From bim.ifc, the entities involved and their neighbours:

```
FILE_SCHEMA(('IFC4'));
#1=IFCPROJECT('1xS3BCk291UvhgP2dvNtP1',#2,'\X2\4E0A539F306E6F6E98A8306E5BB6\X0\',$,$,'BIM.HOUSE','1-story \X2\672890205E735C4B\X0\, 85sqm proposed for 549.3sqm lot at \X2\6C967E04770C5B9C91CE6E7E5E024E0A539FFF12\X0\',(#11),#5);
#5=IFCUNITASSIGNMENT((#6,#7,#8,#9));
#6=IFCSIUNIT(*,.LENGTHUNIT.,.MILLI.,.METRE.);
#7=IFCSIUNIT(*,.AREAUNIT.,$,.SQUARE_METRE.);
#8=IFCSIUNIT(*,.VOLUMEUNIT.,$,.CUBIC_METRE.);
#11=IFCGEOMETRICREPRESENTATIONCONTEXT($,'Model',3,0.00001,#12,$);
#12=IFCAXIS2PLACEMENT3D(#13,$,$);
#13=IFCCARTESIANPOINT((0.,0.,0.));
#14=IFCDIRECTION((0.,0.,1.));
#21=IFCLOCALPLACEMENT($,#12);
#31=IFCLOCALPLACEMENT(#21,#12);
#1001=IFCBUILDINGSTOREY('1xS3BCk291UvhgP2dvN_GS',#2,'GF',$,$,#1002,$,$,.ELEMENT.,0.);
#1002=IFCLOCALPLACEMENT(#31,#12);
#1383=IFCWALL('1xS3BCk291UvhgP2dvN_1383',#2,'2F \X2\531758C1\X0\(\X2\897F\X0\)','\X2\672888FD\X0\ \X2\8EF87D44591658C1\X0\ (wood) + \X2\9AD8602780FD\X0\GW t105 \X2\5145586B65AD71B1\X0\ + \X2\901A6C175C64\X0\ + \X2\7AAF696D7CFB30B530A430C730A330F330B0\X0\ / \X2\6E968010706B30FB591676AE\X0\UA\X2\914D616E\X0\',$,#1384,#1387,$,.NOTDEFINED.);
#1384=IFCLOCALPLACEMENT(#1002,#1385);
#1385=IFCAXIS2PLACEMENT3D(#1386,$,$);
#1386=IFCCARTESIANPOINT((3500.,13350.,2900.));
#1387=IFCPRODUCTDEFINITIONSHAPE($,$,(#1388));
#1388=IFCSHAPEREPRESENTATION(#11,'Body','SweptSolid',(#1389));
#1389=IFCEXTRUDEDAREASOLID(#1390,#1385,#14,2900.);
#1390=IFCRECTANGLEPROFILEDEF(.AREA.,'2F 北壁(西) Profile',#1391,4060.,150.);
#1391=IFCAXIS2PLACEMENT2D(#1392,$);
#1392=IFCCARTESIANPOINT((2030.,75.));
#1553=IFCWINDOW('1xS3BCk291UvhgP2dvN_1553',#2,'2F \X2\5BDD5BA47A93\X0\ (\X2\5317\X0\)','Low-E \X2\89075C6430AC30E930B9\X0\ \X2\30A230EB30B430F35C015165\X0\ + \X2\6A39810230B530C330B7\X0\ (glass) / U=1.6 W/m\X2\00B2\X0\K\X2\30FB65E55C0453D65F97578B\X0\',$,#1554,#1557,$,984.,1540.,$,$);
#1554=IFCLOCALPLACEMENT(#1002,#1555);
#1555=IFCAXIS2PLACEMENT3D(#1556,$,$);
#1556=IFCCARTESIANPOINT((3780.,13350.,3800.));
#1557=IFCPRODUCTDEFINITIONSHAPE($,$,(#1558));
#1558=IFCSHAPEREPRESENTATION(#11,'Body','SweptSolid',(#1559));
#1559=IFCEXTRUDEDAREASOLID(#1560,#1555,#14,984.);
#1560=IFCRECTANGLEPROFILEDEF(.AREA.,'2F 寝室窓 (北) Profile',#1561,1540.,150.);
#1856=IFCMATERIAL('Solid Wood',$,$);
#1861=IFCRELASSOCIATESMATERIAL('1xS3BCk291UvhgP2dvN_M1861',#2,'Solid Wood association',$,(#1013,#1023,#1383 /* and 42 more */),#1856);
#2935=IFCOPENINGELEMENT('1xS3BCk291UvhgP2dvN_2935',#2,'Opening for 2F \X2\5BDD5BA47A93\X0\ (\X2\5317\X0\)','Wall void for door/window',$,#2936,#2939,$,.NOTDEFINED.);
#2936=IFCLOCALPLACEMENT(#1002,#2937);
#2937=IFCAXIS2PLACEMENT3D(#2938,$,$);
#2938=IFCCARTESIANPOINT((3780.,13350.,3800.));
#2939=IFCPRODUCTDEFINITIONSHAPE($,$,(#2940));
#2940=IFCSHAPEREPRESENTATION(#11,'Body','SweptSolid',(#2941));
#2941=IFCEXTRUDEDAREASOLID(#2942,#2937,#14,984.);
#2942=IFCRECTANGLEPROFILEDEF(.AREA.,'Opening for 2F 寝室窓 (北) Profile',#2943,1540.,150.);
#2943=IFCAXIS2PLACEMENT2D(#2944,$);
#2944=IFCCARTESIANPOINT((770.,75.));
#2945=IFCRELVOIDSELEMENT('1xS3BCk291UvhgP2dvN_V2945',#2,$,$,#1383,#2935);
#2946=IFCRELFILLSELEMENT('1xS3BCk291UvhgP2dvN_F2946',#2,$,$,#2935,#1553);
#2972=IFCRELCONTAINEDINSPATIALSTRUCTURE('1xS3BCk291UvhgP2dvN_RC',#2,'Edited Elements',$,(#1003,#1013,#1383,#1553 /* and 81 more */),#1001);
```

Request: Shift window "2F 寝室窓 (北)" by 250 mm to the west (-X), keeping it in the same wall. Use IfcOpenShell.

```python
import ifcopenshell
import ifcopenshell.api.geometry
import ifcopenshell.util.placement
import ifcopenshell.util.unit

model = ifcopenshell.open("bim.ifc")
unit_scale = ifcopenshell.util.unit.calculate_unit_scale(model)

window = model.by_guid("1xS3BCk291UvhgP2dvN_1553")
opening = window.FillsVoids[0].RelatingOpeningElement
wall = opening.VoidsElements[0].RelatingBuildingElement

wall_matrix = ifcopenshell.util.placement.get_local_placement(wall.ObjectPlacement)
shift = wall_matrix[:3, 0] * -0.25 / unit_scale
before = ifcopenshell.util.placement.get_local_placement(window.ObjectPlacement)[:3, 3].copy()

# The window is not placed relative to its opening, so move both.
for product in (opening, window):
    matrix = ifcopenshell.util.placement.get_local_placement(product.ObjectPlacement)
    matrix[:3, 3] += shift
    ifcopenshell.api.geometry.edit_object_placement(model, product=product, matrix=matrix, is_si=False)

after = ifcopenshell.util.placement.get_local_placement(window.ObjectPlacement)[:3, 3]
print("window moved by", (after - before).round(3) + 0.0)

model.write("bim_rev.ifc")
```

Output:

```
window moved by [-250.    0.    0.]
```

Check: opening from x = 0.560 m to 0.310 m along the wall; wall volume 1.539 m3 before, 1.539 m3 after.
